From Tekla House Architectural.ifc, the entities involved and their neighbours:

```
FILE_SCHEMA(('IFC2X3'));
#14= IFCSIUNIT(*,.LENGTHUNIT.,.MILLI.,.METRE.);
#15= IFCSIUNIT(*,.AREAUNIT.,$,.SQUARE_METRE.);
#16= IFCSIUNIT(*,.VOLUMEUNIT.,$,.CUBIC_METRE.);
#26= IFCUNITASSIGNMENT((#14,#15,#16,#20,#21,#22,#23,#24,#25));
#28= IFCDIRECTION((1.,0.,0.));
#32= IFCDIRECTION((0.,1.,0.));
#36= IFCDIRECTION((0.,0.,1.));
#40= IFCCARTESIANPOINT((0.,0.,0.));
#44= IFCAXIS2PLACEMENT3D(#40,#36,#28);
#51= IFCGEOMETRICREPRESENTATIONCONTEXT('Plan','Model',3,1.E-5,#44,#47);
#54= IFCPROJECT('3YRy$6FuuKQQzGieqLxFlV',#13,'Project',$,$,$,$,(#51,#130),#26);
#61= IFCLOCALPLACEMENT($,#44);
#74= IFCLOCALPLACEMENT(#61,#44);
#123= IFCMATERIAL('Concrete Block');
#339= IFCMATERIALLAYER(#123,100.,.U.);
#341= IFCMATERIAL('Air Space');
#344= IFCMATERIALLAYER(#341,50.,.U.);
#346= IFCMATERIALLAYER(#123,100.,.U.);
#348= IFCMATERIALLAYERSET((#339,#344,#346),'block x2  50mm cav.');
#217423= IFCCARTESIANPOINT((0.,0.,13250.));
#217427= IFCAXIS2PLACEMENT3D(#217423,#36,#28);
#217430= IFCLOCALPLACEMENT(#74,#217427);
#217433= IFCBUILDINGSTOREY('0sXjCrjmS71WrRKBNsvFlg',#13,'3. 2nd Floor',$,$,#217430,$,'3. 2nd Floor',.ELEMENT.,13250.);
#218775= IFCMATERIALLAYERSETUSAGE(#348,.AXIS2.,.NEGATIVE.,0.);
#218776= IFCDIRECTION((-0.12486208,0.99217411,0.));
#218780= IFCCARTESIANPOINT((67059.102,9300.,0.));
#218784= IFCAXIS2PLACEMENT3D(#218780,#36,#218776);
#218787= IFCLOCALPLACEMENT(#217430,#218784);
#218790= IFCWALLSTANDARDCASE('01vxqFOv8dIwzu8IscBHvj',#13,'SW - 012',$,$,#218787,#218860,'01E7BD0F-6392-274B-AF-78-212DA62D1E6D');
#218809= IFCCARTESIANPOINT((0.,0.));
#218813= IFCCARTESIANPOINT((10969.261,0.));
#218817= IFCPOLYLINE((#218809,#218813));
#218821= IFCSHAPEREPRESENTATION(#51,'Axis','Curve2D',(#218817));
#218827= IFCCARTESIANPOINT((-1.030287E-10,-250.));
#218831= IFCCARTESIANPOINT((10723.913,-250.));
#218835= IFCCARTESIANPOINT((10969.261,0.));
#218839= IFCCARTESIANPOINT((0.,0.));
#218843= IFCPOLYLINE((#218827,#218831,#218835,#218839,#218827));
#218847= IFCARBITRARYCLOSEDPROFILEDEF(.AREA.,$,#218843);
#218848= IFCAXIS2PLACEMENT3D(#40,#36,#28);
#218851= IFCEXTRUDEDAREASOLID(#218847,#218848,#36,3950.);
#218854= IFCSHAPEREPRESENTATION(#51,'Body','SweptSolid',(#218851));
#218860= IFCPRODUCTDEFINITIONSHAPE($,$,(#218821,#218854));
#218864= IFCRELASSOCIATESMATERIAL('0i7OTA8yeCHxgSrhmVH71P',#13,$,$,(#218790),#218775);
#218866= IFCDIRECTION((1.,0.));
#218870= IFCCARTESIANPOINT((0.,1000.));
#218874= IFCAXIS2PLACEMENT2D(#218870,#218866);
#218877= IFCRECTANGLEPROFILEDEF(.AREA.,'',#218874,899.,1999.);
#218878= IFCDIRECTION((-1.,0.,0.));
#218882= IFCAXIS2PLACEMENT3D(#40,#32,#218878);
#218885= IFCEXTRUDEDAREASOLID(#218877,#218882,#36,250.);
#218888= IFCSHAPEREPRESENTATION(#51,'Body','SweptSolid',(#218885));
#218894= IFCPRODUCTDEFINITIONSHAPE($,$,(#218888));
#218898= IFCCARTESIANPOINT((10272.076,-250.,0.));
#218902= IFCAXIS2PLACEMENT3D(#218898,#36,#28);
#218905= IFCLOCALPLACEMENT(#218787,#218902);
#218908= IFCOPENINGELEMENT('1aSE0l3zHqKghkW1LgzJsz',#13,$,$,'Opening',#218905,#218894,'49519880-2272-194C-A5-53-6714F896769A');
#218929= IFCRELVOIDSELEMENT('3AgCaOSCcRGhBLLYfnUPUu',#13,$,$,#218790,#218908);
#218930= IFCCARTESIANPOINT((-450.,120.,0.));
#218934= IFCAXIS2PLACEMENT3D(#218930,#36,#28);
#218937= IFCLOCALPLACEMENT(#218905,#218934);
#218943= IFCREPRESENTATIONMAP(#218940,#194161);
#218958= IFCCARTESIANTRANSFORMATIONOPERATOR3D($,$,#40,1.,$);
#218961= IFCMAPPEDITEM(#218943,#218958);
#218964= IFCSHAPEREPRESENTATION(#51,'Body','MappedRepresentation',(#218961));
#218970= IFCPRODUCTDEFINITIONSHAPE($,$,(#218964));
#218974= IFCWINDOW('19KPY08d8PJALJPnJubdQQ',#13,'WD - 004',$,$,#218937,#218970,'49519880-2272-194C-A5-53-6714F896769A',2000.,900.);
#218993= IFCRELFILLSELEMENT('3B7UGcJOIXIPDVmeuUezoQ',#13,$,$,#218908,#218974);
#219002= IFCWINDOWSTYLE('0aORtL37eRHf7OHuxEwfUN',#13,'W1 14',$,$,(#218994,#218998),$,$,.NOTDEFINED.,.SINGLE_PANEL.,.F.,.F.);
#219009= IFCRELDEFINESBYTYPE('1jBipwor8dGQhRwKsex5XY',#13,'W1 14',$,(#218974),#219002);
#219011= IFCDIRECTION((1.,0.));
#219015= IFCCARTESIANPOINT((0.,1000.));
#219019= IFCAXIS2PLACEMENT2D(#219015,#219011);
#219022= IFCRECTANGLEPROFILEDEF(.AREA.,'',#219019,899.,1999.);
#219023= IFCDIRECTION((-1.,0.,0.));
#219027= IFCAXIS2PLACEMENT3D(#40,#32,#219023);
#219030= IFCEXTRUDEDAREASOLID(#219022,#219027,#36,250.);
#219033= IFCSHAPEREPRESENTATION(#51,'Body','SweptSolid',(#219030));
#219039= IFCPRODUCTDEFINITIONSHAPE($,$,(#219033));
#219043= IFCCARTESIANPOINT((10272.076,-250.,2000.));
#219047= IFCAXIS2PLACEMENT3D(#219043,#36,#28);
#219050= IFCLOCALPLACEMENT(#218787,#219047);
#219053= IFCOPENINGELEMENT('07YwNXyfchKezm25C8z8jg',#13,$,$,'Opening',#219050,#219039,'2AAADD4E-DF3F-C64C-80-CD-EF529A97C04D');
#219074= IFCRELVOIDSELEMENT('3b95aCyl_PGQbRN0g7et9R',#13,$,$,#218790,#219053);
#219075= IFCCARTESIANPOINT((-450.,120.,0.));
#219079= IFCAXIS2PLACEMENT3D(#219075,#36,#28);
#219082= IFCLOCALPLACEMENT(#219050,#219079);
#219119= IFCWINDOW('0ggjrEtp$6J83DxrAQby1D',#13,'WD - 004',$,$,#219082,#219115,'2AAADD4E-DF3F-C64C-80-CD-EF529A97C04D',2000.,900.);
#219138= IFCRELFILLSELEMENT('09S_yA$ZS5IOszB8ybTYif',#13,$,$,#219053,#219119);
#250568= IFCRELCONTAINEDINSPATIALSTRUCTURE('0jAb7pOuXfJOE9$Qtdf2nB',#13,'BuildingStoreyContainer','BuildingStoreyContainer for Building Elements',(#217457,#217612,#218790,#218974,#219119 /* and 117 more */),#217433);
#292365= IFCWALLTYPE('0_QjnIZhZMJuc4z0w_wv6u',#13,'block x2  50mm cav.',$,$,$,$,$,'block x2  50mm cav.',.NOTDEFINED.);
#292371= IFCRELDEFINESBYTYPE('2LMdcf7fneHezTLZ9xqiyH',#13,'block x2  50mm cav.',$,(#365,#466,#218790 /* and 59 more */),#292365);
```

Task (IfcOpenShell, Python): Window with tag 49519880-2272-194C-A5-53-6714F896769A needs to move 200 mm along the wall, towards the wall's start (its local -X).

```python
import ifcopenshell
import ifcopenshell.api.geometry
import ifcopenshell.util.placement

model = ifcopenshell.open("Tekla House Architectural.ifc")

window = model.by_guid("19KPY08d8PJALJPnJubdQQ")
opening = window.FillsVoids[0].RelatingOpeningElement
wall = opening.VoidsElements[0].RelatingBuildingElement

wall_matrix = ifcopenshell.util.placement.get_local_placement(wall.ObjectPlacement)
shift = wall_matrix[:3, 0] * -200.0
before = ifcopenshell.util.placement.get_local_placement(window.ObjectPlacement)[:3, 3].copy()

# The window is placed relative to its opening, so it follows when the opening moves.
matrix = ifcopenshell.util.placement.get_local_placement(opening.ObjectPlacement)
matrix[:3, 3] += shift
ifcopenshell.api.geometry.edit_object_placement(
    model, product=opening, matrix=matrix, is_si=False, should_transform_children=True
)

after = ifcopenshell.util.placement.get_local_placement(window.ObjectPlacement)[:3, 3]
print("window moved by", (after - before).round(3) + 0.0)

model.write("Tekla House Architectural_edited.ifc")
```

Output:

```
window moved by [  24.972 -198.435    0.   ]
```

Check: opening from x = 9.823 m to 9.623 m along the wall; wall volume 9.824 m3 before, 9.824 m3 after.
